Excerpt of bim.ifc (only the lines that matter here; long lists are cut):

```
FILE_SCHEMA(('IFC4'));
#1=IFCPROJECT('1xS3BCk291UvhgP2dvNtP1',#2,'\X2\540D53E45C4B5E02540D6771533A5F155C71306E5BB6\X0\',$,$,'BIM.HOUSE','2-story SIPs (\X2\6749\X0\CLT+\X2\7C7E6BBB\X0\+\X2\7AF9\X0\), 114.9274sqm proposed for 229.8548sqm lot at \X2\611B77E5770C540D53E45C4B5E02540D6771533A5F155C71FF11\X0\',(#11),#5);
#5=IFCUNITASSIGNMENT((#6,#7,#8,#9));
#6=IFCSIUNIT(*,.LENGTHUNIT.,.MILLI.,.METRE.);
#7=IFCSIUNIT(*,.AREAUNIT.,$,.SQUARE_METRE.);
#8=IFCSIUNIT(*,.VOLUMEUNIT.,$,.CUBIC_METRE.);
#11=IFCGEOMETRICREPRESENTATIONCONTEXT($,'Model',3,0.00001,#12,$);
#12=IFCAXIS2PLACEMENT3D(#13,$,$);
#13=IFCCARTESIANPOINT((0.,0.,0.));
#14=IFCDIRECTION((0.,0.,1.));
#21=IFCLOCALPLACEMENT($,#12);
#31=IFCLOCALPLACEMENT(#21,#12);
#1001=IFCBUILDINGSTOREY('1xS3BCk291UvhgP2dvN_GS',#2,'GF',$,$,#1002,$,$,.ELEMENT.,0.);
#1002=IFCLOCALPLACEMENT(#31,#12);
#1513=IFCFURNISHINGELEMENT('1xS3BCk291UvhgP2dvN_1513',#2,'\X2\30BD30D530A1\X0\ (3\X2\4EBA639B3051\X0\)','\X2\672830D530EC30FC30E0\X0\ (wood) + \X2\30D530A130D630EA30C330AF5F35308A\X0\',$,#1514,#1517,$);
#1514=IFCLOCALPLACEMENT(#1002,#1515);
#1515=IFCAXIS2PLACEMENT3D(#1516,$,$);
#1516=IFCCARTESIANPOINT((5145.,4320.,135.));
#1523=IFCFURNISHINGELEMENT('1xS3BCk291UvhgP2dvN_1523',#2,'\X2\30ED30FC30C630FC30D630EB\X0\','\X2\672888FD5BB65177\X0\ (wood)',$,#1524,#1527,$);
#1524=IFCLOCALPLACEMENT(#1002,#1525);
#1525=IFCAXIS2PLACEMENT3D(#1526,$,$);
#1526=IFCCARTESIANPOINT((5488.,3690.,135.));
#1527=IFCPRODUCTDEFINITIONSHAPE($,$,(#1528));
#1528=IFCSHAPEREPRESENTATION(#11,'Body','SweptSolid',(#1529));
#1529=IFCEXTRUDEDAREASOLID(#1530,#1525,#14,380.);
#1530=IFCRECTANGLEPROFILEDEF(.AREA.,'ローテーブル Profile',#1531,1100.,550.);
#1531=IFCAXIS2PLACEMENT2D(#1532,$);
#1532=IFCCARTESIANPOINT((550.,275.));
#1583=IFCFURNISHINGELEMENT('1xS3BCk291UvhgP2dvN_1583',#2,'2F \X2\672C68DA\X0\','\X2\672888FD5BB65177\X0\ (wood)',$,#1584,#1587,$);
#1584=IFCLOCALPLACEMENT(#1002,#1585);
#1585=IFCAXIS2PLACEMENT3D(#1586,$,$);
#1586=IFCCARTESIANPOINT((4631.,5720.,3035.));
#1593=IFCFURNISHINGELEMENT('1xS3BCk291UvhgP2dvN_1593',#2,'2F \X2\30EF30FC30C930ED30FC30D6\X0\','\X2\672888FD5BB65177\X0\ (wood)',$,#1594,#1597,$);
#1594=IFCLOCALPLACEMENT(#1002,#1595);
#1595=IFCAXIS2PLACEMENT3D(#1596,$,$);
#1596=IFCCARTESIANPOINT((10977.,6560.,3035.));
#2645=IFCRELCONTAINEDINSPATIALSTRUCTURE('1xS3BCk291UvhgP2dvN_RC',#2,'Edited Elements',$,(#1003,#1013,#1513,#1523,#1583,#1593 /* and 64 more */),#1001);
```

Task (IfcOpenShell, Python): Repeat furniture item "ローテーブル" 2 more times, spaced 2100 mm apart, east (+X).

```python
import numpy as np
import ifcopenshell
import ifcopenshell.api.geometry
import ifcopenshell.api.root
import ifcopenshell.util.element
import ifcopenshell.util.placement
import ifcopenshell.util.unit

model = ifcopenshell.open("bim.ifc")
unit_scale = ifcopenshell.util.unit.calculate_unit_scale(model)


def reuse_history(source, copy):
    """copy_class also copies each property set's owner history, people and application; keep the originals."""
    for rel in copy.IsDefinedBy:
        if rel.is_a("IfcRelDefinesByProperties") and (history := rel.RelatingPropertyDefinition.OwnerHistory):
            rel.RelatingPropertyDefinition.OwnerHistory = source.OwnerHistory
            ifcopenshell.util.element.remove_deep2(model, history)


source = model.by_id(1523)
base = ifcopenshell.util.placement.get_local_placement(source.ObjectPlacement)
step = np.array([1.0, 0.0, 0.0]) * 2.1 / unit_scale

for i in range(1, 3):
    copy = ifcopenshell.api.root.copy_class(model, product=source)
    copy.Representation = ifcopenshell.util.element.copy_deep(
        model, source.Representation, exclude=["IfcGeometricRepresentationContext", "IfcRepresentationMap"]
    )
    reuse_history(source, copy)
    matrix = base.copy()
    matrix[:3, 3] += i * step
    print("added at", matrix[:3, 3].round(3) + 0.0)
    ifcopenshell.api.geometry.edit_object_placement(model, product=copy, matrix=matrix, is_si=False)

model.write("bim_v2.ifc")
```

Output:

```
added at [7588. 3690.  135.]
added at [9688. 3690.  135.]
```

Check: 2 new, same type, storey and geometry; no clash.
